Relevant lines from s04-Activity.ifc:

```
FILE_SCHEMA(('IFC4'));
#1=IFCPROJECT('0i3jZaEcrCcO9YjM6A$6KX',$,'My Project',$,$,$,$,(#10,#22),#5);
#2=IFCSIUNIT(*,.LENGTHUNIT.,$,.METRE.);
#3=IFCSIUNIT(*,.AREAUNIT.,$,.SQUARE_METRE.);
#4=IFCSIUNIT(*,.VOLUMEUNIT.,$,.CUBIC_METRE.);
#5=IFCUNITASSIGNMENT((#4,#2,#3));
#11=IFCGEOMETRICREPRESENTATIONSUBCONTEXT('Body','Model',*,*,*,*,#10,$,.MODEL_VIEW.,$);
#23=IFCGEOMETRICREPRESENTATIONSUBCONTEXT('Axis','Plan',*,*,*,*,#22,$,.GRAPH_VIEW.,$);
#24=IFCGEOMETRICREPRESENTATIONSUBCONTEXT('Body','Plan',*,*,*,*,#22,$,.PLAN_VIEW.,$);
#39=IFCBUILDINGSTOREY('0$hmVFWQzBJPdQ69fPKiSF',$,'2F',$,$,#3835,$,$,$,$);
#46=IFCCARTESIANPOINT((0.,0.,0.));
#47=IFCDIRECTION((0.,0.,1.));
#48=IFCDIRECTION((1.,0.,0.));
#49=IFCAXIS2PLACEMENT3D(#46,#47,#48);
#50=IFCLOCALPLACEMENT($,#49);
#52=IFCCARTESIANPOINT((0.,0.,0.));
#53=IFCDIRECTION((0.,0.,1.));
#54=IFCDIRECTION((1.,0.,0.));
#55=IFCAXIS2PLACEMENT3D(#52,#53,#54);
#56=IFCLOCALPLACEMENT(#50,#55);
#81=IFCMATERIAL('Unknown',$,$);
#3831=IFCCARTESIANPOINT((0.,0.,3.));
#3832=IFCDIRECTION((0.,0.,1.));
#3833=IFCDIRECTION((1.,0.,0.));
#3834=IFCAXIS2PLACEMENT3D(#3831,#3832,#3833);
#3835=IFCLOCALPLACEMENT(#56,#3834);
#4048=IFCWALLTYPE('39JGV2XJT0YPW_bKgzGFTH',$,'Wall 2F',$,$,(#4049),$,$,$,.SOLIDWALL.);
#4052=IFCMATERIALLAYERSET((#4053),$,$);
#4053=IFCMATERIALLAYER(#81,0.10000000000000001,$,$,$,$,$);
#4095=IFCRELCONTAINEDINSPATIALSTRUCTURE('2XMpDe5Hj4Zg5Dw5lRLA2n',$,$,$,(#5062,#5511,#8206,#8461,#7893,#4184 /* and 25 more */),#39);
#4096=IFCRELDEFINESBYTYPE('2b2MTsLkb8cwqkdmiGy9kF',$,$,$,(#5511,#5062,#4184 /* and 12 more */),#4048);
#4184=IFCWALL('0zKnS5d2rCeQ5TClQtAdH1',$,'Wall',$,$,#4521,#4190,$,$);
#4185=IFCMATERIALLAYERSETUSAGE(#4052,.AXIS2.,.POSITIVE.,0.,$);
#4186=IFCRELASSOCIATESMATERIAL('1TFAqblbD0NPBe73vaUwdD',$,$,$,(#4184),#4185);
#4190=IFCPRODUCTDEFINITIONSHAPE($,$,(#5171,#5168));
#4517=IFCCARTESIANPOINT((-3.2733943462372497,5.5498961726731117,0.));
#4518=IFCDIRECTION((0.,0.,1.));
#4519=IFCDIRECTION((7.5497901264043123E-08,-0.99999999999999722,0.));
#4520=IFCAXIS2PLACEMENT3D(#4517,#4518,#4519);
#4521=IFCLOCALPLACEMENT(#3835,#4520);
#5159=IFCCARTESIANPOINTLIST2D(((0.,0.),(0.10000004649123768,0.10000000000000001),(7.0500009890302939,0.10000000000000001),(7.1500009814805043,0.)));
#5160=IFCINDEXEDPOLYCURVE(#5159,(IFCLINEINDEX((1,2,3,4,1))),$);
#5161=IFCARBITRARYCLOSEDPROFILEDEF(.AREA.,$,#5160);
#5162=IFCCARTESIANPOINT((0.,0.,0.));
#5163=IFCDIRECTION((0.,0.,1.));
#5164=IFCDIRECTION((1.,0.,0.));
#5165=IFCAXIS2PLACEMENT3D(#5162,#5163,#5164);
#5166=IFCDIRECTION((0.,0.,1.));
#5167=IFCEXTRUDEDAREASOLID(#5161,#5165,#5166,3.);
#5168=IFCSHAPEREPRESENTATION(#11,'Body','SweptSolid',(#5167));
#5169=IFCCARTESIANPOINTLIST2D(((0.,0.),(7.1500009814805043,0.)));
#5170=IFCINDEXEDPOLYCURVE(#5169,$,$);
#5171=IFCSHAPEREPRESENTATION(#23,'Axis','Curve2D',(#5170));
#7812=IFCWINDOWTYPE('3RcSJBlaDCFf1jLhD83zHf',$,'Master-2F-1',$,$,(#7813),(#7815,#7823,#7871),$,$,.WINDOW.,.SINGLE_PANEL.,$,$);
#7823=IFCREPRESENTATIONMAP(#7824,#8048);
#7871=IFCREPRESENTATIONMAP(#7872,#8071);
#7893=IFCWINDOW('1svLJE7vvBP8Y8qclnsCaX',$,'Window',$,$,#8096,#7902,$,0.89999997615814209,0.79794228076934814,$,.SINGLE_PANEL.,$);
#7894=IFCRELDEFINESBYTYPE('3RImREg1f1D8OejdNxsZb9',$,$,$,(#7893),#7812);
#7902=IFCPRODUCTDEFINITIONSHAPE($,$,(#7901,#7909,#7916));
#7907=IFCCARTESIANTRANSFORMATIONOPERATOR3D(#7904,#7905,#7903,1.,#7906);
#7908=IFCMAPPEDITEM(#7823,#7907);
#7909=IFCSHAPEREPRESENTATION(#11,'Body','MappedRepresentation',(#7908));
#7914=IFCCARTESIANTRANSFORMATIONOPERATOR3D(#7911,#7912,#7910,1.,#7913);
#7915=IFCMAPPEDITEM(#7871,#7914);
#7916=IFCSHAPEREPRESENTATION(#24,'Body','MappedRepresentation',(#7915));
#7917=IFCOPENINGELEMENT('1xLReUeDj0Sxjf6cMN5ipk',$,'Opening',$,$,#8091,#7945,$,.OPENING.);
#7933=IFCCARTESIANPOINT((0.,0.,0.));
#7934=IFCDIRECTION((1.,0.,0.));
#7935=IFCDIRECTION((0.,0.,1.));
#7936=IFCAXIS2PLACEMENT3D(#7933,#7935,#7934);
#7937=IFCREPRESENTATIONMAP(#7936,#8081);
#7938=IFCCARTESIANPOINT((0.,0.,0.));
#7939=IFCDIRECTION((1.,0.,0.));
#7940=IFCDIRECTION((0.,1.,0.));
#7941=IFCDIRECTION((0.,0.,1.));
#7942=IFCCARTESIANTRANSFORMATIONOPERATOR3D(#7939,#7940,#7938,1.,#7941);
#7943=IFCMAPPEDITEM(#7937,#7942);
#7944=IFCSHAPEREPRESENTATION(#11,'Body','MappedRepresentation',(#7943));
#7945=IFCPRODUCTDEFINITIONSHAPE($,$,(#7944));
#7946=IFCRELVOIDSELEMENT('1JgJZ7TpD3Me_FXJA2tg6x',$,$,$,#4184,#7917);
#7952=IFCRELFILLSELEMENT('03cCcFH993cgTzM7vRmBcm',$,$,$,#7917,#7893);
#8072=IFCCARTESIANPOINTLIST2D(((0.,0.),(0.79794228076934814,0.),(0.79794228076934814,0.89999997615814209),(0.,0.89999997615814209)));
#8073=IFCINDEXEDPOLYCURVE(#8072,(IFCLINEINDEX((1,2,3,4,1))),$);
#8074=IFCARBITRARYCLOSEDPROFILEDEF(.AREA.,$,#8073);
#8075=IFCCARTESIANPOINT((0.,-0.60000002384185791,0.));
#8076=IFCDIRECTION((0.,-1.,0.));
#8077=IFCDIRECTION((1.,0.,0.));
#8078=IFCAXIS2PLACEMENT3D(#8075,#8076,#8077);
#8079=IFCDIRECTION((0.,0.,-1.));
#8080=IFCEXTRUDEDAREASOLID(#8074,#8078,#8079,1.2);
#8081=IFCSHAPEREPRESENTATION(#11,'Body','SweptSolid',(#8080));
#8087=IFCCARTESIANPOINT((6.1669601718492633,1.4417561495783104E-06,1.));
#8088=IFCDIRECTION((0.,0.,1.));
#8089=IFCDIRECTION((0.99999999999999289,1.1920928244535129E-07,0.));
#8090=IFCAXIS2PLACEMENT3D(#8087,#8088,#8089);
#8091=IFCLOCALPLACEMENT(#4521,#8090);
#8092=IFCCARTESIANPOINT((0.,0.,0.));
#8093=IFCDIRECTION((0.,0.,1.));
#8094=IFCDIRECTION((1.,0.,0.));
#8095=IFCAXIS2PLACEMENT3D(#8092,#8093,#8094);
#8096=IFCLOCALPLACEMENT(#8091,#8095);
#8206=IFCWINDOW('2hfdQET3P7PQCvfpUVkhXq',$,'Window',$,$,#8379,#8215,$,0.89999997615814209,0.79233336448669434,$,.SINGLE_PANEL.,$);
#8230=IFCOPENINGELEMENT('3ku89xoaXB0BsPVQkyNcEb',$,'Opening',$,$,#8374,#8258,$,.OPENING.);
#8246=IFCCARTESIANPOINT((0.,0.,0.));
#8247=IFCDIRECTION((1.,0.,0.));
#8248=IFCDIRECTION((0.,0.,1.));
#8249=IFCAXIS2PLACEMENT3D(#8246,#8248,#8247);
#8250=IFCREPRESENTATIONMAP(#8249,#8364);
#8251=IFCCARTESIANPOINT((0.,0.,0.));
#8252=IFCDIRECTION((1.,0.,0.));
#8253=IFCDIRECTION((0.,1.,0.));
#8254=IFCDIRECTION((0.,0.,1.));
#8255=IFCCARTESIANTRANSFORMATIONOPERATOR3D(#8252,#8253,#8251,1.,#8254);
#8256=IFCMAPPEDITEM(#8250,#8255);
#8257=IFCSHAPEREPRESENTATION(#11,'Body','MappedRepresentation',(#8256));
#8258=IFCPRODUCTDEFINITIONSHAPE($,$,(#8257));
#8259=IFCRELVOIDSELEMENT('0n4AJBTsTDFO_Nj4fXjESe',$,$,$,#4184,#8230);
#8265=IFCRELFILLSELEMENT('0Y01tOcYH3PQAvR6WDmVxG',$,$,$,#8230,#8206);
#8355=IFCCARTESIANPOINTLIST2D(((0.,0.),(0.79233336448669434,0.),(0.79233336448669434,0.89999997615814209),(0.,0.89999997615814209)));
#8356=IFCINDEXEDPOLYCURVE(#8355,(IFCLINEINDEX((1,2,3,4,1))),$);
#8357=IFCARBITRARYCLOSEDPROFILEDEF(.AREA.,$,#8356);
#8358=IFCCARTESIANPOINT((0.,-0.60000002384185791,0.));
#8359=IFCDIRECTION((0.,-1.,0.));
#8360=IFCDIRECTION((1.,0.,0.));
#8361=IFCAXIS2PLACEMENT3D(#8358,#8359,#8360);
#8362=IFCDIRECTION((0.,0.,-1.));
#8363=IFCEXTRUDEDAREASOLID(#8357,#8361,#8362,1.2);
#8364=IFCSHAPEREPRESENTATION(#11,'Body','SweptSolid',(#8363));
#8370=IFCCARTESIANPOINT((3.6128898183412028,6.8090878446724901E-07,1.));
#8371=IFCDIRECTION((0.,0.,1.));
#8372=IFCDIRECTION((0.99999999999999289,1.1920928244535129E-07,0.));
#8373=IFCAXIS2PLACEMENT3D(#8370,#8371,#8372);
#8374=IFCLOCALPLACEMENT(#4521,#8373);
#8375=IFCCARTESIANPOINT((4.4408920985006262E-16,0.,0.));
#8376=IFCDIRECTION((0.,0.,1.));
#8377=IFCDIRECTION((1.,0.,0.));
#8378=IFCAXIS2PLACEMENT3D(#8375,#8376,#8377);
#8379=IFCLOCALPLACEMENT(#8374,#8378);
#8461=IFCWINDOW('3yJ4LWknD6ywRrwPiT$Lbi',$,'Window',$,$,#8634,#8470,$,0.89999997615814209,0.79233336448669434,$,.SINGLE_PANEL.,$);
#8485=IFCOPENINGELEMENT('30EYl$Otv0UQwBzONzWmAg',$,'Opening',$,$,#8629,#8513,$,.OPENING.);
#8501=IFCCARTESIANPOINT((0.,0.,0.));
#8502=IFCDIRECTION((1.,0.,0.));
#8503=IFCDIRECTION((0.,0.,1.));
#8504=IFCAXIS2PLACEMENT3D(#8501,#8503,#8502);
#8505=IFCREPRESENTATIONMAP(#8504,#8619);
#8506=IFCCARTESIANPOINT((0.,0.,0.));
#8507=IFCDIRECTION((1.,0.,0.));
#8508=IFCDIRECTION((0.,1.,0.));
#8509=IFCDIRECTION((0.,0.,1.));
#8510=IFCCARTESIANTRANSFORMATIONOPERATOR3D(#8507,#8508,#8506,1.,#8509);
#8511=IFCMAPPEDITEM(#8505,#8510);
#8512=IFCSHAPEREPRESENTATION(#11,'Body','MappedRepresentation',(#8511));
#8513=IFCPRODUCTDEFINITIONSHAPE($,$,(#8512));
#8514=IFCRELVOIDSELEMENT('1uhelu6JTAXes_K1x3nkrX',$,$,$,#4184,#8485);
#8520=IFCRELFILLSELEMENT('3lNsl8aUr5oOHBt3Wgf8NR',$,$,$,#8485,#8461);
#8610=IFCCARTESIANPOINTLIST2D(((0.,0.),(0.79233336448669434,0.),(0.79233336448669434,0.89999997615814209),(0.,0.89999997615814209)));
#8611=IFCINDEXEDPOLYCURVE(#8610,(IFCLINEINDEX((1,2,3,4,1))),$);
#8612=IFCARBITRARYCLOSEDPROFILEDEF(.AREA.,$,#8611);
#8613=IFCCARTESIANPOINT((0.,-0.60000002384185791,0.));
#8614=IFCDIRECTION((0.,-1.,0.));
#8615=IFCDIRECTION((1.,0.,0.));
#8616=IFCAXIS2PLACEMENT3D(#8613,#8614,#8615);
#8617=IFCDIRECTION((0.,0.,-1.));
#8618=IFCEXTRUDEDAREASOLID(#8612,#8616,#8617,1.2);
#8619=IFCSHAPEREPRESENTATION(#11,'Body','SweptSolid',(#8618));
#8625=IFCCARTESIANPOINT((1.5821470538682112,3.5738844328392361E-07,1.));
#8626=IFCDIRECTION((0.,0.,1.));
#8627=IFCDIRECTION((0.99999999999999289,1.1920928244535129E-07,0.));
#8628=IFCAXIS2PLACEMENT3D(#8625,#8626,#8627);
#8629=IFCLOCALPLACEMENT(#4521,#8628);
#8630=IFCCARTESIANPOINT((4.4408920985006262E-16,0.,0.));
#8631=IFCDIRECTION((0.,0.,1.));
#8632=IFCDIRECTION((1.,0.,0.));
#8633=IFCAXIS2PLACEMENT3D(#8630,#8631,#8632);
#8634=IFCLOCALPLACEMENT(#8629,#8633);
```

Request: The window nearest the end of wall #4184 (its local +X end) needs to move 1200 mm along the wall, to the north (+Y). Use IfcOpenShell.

```python
import ifcopenshell
import ifcopenshell.api.geometry
import ifcopenshell.util.placement

model = ifcopenshell.open("s04-Activity.ifc")

window = model.by_guid("1svLJE7vvBP8Y8qclnsCaX")
opening = window.FillsVoids[0].RelatingOpeningElement
wall = opening.VoidsElements[0].RelatingBuildingElement

wall_matrix = ifcopenshell.util.placement.get_local_placement(wall.ObjectPlacement)
shift = wall_matrix[:3, 0] * -1.2
before = ifcopenshell.util.placement.get_local_placement(window.ObjectPlacement)[:3, 3].copy()

# The window is placed relative to its opening, so it follows when the opening moves.
matrix = ifcopenshell.util.placement.get_local_placement(opening.ObjectPlacement)
matrix[:3, 3] += shift
ifcopenshell.api.geometry.edit_object_placement(
    model, product=opening, matrix=matrix, is_si=False, should_transform_children=True
)

after = ifcopenshell.util.placement.get_local_placement(window.ObjectPlacement)[:3, 3]
print("window moved by", (after - before).round(3) + 0.0)

model.write("s04-Activity_rev.ifc")
```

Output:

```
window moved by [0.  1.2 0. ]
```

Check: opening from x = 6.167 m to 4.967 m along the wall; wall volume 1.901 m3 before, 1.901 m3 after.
